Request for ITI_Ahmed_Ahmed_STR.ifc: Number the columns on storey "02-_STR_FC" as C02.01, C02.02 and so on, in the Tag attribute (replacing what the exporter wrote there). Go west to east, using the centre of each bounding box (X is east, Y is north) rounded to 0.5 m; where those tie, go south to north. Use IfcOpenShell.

First a look at what the model holds.

```python
import ifcopenshell
import ifcopenshell.util.element
import ifcopenshell.util.placement

model = ifcopenshell.open("ITI_Ahmed_Ahmed_STR.ifc")
print(model.schema)
storey = next(s for s in model.by_type("IfcBuildingStorey") if s.Name == "02-_STR_FC")
columns = [e for e in ifcopenshell.util.element.get_decomposition(storey) if e.is_a("IfcColumn")]
for e in sorted(columns, key=lambda e: e.id()):
    origin = ifcopenshell.util.placement.get_local_placement(e.ObjectPlacement)[:3, 3]
    print(e.id(), e.Tag, e.Name, origin.round(2) + 0.0, sep=" | ")
```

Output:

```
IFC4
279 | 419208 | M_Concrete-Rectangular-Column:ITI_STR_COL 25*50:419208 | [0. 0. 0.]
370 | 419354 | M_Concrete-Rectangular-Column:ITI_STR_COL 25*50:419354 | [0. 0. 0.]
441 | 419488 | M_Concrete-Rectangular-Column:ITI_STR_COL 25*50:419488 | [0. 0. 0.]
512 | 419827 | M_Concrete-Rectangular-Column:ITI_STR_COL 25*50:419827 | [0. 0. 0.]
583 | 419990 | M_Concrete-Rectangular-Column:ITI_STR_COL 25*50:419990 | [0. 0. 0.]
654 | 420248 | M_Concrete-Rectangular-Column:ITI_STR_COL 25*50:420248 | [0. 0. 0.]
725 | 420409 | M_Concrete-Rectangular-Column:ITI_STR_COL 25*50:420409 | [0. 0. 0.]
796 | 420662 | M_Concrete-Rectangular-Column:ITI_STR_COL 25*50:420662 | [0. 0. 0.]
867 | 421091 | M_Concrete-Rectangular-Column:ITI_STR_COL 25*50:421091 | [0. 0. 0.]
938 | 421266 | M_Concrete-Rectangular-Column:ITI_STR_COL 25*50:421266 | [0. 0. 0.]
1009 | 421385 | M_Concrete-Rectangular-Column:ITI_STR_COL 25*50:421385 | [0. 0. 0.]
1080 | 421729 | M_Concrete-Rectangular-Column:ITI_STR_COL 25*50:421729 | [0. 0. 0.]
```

```python
import ifcopenshell
import ifcopenshell.geom
import ifcopenshell.util.element
import ifcopenshell.util.shape

model = ifcopenshell.open("ITI_Ahmed_Ahmed_STR.ifc")
settings = ifcopenshell.geom.settings()
settings.set("use-world-coords", True)


def centre(element):
    shape = ifcopenshell.geom.create_shape(settings, element)
    return ifcopenshell.util.shape.get_bbox_centroid(shape.geometry)


storey = next(s for s in model.by_type("IfcBuildingStorey") if s.Name == "02-_STR_FC")
columns = [e for e in ifcopenshell.util.element.get_decomposition(storey) if e.is_a("IfcColumn")]

# Insertion points can sit at a corner or the storey origin, so sort by the geometry (in metres).
centres = {e: centre(e) for e in columns}
columns.sort(key=lambda e: (round(centres[e][0] / 0.5), centres[e][1]))

for i, e in enumerate(columns, start=1):
    number = f"C02.{i:02d}"
    e.Tag = number
    print(e.id(), number)

model.write("ITI_Ahmed_Ahmed_STR_v2.ifc")
```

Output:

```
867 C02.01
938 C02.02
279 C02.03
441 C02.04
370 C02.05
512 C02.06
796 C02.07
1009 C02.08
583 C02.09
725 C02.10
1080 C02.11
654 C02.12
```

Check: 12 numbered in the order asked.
